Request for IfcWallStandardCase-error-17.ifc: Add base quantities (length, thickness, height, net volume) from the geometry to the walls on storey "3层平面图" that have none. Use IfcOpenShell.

First a look at what the model holds.

```python
import ifcopenshell
import ifcopenshell.util.element
import ifcopenshell.util.unit

model = ifcopenshell.open("IfcWallStandardCase-error-17.ifc")
print(model.schema)
for unit_type in ("LENGTHUNIT", "AREAUNIT", "VOLUMEUNIT"):
    print(unit_type, ifcopenshell.util.unit.calculate_unit_scale(model, unit_type))
storey = next(s for s in model.by_type("IfcBuildingStorey") if s.Name == "3层平面图")
walls = [e for e in ifcopenshell.util.element.get_decomposition(storey) if e.is_a("IfcWall")]
for e in sorted(walls, key=lambda e: e.id()):
    print(e.id(), e.is_a(), e.Name, list(ifcopenshell.util.element.get_psets(e, qtos_only=True)), sep=" | ")
```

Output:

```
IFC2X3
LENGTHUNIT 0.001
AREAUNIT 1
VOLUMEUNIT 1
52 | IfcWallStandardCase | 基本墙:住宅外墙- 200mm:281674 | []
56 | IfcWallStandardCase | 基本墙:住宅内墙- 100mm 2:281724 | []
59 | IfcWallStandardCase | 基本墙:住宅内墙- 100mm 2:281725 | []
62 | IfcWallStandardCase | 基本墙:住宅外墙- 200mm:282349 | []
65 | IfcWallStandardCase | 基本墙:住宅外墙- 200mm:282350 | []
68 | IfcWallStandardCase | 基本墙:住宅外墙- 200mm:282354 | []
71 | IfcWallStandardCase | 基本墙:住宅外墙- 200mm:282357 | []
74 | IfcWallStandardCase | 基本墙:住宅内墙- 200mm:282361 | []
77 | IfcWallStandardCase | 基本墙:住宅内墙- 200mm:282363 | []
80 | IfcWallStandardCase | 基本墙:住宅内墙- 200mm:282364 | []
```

```python
import ifcopenshell
import ifcopenshell.api.pset
import ifcopenshell.geom
import ifcopenshell.util.element
import ifcopenshell.util.shape
import ifcopenshell.util.unit

model = ifcopenshell.open("IfcWallStandardCase-error-17.ifc")
unit_scale = ifcopenshell.util.unit.calculate_unit_scale(model)
volume_scale = ifcopenshell.util.unit.calculate_unit_scale(model, "VOLUMEUNIT")
settings = ifcopenshell.geom.settings()

storey = next(s for s in model.by_type("IfcBuildingStorey") if s.Name == "3层平面图")
walls = [e for e in ifcopenshell.util.element.get_decomposition(storey) if e.is_a("IfcWall")]

for e in sorted(walls, key=lambda e: e.id()):
    if ifcopenshell.util.element.get_psets(e, qtos_only=True, should_inherit=False):
        continue
    # Geometry comes back in metres, in the element's own axes.
    shape = ifcopenshell.geom.create_shape(settings, e)
    values = {
        "Length": ifcopenshell.util.shape.get_x(shape.geometry) / unit_scale,
        "Width": ifcopenshell.util.shape.get_y(shape.geometry) / unit_scale,
        "Height": ifcopenshell.util.shape.get_z(shape.geometry) / unit_scale,
        "NetVolume": ifcopenshell.util.shape.get_volume(shape.geometry) / volume_scale,
    }
    qto = ifcopenshell.api.pset.add_qto(model, product=e, name="BaseQuantities")
    ifcopenshell.api.pset.edit_qto(model, qto=qto, properties=values)
    print(e.id(), {k: round(v, 3) for k, v in values.items()})

model.write("IfcWallStandardCase-error-17_rev.ifc")
```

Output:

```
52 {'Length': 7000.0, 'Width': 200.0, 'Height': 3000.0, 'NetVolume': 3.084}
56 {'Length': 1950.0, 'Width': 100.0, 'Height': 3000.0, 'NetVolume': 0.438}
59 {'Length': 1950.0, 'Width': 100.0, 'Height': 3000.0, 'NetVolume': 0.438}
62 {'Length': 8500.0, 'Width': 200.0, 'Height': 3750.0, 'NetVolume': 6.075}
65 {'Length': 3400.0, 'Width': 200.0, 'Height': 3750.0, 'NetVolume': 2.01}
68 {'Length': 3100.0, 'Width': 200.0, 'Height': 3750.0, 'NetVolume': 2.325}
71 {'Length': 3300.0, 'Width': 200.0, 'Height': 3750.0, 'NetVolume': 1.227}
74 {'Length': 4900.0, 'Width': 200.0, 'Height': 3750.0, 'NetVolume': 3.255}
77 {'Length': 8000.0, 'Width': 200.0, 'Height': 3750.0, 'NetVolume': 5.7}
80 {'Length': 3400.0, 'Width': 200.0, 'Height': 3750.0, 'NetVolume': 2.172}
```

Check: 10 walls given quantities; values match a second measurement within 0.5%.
